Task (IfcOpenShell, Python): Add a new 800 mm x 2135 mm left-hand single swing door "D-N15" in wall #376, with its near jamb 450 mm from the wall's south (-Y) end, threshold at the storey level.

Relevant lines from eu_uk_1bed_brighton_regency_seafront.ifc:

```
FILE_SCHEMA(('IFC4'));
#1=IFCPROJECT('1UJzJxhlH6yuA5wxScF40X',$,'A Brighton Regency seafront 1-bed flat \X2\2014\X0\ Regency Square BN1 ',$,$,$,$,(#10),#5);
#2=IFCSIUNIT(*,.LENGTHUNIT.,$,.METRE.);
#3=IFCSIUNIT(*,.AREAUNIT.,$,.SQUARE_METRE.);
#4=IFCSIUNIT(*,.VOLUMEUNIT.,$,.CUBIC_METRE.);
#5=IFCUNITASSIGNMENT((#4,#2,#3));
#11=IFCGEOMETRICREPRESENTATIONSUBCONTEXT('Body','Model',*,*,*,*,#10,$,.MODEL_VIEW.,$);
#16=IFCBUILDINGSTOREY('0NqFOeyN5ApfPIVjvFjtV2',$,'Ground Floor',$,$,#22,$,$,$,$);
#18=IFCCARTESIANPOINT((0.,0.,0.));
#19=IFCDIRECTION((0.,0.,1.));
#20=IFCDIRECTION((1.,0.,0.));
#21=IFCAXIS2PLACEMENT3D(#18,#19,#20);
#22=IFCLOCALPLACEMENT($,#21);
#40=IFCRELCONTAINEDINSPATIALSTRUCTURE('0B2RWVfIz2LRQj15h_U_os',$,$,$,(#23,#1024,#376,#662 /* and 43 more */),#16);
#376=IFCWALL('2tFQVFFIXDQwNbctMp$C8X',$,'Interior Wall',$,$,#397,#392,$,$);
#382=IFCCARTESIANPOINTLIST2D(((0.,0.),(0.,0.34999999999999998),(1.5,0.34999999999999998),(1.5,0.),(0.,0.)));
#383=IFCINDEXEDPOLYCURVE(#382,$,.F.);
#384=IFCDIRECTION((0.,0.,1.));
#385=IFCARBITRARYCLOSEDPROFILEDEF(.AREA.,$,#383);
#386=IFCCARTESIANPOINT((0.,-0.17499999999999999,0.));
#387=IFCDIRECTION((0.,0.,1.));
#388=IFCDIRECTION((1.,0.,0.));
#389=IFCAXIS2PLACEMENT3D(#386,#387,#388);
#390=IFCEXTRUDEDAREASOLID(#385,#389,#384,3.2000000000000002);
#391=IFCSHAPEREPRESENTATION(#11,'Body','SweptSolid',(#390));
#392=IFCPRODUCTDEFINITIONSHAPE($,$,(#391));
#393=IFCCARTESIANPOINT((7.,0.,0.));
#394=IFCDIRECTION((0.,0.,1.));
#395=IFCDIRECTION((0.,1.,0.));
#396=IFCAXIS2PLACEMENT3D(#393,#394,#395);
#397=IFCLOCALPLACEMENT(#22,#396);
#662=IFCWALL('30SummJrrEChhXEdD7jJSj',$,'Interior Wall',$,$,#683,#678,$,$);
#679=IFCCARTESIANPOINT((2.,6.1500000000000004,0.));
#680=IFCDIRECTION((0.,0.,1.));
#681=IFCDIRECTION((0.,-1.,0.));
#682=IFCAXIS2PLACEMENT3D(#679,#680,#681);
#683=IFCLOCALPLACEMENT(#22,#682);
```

```python
import numpy as np
import ifcopenshell
import ifcopenshell.api.feature
import ifcopenshell.api.geometry
import ifcopenshell.api.root
import ifcopenshell.api.spatial
import ifcopenshell.geom
import ifcopenshell.util.element
import ifcopenshell.util.placement
import ifcopenshell.util.representation
import ifcopenshell.util.shape
import ifcopenshell.util.unit

model = ifcopenshell.open("eu_uk_1bed_brighton_regency_seafront.ifc")
unit_scale = ifcopenshell.util.unit.calculate_unit_scale(model)
settings = ifcopenshell.geom.settings()


def volume(element):
    """Net volume in cubic metres, openings subtracted."""
    shape = ifcopenshell.geom.create_shape(settings, element)
    return ifcopenshell.util.shape.get_volume(shape.geometry)


wall = model.by_id(376)
storey = ifcopenshell.util.element.get_container(wall, ifc_class="IfcBuildingStorey")
context = ifcopenshell.util.representation.get_context(model, "Model", "Body", "MODEL_VIEW")
before = volume(wall)

width, height, from_end, sill = 0.8, 2.135, 0.45, 0.0  # metres

# The wall runs along its own X axis, and the end named is its -X end.
wall_shape = ifcopenshell.geom.create_shape(settings, wall)
x, y, z = ifcopenshell.util.shape.get_vertices(wall_shape.geometry).T
start = x.min() + from_end
face, thickness = float(y.min()), float(y.max() - y.min())
wall_matrix = ifcopenshell.util.placement.get_local_placement(wall.ObjectPlacement)
level = ifcopenshell.util.placement.get_local_placement(storey.ObjectPlacement)[2, 3]


def in_wall(x, y):
    """Placement at x, y metres in the wall's axes, at sill height."""
    matrix = wall_matrix.copy()
    matrix[:, 3] = wall_matrix @ np.array([x / unit_scale, y / unit_scale, 0.0, 1.0])
    matrix[2, 3] = level + sill / unit_scale
    return matrix


# Opening: a box that overshoots both wall faces by 50 mm.
opening = ifcopenshell.api.root.create_entity(model, ifc_class="IfcOpeningElement", predefined_type="OPENING")
box = ifcopenshell.api.geometry.add_wall_representation(
    model, context=context, length=width, height=height, thickness=thickness + 0.1
)
ifcopenshell.api.geometry.assign_representation(model, product=opening, representation=box)
ifcopenshell.api.geometry.edit_object_placement(model, product=opening, matrix=in_wall(start, face - 0.05), is_si=False)
ifcopenshell.api.feature.add_feature(model, feature=opening, element=wall)

door = ifcopenshell.api.root.create_entity(model, ifc_class="IfcDoor", name="D-N15", predefined_type="DOOR")
door.OverallWidth, door.OverallHeight = width / unit_scale, height / unit_scale
door.OperationType = "SINGLE_SWING_LEFT"
body = ifcopenshell.api.geometry.add_door_representation(
    model,
    context=context,
    overall_width=door.OverallWidth,
    overall_height=door.OverallHeight,
    operation_type="SINGLE_SWING_LEFT",
    lining_properties={"LiningDepth": thickness / unit_scale, "ThresholdDepth": thickness / unit_scale},
)
ifcopenshell.api.geometry.assign_representation(model, product=door, representation=body)
ifcopenshell.api.spatial.assign_container(model, products=[door], relating_structure=storey)
ifcopenshell.api.feature.add_filling(model, opening=opening, element=door)

# The lining spans the wall, so the door starts at the wall face.
ifcopenshell.api.geometry.edit_object_placement(model, product=door, matrix=in_wall(start, face), is_si=False)

after = volume(wall)

print(f"wall volume {before:.3f} -> {after:.3f} m3")

model.write("eu_uk_1bed_brighton_regency_seafront-out.ifc")
```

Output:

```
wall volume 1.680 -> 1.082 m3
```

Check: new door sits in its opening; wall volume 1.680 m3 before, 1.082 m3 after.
